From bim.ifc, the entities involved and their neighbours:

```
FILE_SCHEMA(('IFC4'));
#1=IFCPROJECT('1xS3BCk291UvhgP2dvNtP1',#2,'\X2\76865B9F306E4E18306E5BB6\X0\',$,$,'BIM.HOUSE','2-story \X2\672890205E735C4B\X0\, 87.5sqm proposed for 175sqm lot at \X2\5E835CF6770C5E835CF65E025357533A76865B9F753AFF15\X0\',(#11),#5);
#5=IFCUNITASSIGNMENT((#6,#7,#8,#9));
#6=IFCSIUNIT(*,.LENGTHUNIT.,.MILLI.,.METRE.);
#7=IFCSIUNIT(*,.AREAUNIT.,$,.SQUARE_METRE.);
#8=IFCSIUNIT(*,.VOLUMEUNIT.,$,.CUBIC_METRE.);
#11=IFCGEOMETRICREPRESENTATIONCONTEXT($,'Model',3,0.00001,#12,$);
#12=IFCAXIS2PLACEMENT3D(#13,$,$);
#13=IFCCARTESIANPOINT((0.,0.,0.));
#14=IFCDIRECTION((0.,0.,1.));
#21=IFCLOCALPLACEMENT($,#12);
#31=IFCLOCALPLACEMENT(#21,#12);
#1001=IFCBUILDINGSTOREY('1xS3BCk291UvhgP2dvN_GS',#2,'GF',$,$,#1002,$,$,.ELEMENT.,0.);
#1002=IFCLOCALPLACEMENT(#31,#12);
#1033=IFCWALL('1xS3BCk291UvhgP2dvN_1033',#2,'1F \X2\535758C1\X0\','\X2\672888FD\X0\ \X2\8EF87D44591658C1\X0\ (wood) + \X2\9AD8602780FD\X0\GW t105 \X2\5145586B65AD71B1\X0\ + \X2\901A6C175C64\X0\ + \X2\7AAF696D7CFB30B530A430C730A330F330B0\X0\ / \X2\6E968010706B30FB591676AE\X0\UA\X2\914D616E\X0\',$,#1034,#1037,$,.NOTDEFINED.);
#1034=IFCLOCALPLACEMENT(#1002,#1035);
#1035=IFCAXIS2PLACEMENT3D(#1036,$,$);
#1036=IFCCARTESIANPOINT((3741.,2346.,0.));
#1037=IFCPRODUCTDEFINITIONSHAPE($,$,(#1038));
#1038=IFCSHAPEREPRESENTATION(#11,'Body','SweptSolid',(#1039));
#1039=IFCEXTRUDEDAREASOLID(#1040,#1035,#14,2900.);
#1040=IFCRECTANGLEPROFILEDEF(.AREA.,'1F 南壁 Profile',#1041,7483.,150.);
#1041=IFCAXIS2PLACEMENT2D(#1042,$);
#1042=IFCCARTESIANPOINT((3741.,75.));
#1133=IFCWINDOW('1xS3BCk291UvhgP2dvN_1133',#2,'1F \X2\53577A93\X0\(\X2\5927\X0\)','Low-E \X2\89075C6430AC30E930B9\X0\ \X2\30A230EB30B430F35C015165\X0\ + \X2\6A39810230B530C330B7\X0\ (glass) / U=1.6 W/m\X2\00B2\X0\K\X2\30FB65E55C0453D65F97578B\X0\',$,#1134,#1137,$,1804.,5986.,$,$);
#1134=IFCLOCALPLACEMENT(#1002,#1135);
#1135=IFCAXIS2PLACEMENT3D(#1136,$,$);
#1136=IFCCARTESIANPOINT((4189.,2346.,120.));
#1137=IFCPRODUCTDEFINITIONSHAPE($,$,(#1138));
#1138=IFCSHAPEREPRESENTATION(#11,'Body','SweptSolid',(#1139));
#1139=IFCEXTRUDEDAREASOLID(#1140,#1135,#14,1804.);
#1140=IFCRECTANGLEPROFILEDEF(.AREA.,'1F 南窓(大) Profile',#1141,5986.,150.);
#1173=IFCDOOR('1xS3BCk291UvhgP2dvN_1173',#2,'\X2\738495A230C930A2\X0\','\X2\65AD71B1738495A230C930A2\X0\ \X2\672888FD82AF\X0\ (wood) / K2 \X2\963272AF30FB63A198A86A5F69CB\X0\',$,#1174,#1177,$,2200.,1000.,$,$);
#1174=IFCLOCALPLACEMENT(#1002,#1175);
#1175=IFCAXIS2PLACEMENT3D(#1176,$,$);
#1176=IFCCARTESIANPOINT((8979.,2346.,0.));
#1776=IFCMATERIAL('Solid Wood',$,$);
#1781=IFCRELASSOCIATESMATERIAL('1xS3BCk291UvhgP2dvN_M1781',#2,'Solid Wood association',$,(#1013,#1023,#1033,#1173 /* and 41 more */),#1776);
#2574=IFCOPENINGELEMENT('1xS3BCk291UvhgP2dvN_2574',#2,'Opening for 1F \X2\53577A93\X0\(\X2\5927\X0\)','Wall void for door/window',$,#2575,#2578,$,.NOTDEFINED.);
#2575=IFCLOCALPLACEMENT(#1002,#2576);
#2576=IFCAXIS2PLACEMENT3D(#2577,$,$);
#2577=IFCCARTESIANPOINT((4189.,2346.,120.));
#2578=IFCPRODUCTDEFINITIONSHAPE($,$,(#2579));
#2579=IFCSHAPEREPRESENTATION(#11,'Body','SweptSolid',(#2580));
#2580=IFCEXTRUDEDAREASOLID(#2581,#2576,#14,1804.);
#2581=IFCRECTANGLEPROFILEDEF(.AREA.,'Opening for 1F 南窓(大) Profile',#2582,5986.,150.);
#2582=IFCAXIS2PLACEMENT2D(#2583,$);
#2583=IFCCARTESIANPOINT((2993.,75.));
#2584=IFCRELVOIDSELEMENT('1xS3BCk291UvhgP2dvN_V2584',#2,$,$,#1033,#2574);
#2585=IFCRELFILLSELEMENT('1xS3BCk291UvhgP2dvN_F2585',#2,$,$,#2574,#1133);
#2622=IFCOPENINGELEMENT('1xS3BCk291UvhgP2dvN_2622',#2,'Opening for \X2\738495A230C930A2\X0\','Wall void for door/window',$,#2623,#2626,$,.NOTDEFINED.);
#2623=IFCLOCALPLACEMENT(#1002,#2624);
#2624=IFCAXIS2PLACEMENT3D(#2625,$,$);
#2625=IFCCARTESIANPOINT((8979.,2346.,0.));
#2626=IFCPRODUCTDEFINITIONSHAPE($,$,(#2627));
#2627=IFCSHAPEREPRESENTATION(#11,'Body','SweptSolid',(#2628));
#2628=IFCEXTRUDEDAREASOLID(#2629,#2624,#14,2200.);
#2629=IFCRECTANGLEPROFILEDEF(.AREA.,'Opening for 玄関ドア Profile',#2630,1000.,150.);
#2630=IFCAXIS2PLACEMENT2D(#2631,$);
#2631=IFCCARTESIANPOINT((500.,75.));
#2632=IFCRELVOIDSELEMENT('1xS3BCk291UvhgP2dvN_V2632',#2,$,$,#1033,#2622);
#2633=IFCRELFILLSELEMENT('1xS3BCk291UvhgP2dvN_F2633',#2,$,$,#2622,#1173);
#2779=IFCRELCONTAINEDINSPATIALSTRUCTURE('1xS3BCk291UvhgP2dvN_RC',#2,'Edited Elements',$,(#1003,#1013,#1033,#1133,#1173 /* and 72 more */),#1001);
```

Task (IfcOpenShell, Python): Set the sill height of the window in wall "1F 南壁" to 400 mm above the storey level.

```python
import numpy as np
import ifcopenshell
import ifcopenshell.api.geometry
import ifcopenshell.geom
import ifcopenshell.util.element
import ifcopenshell.util.placement
import ifcopenshell.util.shape
import ifcopenshell.util.unit

model = ifcopenshell.open("bim.ifc")
unit_scale = ifcopenshell.util.unit.calculate_unit_scale(model)

window = model.by_id(1133)
opening = window.FillsVoids[0].RelatingOpeningElement
storey = ifcopenshell.util.element.get_container(window, ifc_class="IfcBuildingStorey")
level = ifcopenshell.util.placement.get_local_placement(storey.ObjectPlacement)[2, 3]

# The opening's origin need not be at the sill, so measure its lowest point.
shape = ifcopenshell.geom.create_shape(ifcopenshell.geom.settings(), opening)
bottom = ifcopenshell.util.shape.get_shape_bottom_elevation(shape, shape.geometry) / unit_scale
dz = level + 400.0 - bottom

shift = np.array([0.0, 0.0, dz])
# The window is not placed relative to its opening, so move both.
for product in (opening, window):
    matrix = ifcopenshell.util.placement.get_local_placement(product.ObjectPlacement)
    matrix[:3, 3] += shift
    ifcopenshell.api.geometry.edit_object_placement(model, product=product, matrix=matrix, is_si=False)

print(f"moved by {dz * unit_scale:+.3f} m")

model.write("bim_rev.ifc")
```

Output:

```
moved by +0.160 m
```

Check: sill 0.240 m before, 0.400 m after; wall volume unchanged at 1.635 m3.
